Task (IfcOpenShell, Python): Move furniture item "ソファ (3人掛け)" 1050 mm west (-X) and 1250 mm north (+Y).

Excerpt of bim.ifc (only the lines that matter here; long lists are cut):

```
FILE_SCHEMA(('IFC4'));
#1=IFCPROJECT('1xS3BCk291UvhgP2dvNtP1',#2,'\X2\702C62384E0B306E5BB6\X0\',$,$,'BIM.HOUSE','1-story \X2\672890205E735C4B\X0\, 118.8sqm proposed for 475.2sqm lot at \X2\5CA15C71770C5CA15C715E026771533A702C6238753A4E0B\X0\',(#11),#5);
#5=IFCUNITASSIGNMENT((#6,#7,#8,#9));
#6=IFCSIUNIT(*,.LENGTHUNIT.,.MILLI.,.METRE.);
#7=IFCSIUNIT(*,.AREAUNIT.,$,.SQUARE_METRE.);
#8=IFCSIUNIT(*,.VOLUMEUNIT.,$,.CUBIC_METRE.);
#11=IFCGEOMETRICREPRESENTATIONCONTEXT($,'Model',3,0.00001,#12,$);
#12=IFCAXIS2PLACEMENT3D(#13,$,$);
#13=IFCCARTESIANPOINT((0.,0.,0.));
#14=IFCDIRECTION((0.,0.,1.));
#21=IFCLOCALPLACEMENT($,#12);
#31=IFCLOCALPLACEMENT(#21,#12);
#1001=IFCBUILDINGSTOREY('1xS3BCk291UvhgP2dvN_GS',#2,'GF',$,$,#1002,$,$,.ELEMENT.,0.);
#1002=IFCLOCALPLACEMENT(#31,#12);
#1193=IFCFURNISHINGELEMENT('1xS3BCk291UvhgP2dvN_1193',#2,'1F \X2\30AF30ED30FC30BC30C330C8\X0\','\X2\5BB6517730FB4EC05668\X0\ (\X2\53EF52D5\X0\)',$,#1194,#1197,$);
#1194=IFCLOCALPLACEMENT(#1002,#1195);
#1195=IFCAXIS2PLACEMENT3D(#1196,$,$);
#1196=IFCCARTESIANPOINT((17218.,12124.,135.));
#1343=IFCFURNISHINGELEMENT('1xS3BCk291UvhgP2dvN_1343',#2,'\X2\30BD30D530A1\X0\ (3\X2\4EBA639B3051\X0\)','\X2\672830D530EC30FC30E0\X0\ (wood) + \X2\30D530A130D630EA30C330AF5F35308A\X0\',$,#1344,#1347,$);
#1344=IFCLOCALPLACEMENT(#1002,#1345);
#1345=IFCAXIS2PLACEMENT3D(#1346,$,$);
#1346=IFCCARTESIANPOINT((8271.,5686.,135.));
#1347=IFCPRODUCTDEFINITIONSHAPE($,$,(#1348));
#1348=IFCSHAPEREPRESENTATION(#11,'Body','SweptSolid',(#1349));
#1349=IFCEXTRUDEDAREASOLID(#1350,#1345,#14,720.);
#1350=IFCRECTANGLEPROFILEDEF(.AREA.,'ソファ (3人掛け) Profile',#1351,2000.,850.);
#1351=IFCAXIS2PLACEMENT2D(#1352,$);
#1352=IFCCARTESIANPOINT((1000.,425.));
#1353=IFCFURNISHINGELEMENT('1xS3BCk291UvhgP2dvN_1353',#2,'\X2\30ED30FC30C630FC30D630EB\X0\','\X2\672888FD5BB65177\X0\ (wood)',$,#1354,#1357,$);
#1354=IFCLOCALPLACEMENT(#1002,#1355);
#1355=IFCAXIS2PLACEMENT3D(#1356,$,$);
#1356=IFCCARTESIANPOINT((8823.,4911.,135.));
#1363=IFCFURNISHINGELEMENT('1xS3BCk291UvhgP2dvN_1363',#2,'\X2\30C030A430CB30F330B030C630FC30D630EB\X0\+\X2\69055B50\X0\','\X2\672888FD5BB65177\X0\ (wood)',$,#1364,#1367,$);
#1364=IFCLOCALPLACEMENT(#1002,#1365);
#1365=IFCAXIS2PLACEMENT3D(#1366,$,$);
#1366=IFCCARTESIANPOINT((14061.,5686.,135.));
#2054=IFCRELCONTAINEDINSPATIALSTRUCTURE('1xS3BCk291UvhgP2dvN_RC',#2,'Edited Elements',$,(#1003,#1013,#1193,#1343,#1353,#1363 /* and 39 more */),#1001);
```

```python
import ifcopenshell
import ifcopenshell.api.geometry
import ifcopenshell.util.placement

model = ifcopenshell.open("bim.ifc")

item = model.by_guid("1xS3BCk291UvhgP2dvN_1343")
matrix = ifcopenshell.util.placement.get_local_placement(item.ObjectPlacement)
matrix[0, 3] -= 1050.0
matrix[1, 3] += 1250.0
ifcopenshell.api.geometry.edit_object_placement(model, product=item, matrix=matrix, is_si=False)

print(ifcopenshell.util.placement.get_local_placement(item.ObjectPlacement).round(3) + 0.0)

model.write("bim_edited.ifc")
```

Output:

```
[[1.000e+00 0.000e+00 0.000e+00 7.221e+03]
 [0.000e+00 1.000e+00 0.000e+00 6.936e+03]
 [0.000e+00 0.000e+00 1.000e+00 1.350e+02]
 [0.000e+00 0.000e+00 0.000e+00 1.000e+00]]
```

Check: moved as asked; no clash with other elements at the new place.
